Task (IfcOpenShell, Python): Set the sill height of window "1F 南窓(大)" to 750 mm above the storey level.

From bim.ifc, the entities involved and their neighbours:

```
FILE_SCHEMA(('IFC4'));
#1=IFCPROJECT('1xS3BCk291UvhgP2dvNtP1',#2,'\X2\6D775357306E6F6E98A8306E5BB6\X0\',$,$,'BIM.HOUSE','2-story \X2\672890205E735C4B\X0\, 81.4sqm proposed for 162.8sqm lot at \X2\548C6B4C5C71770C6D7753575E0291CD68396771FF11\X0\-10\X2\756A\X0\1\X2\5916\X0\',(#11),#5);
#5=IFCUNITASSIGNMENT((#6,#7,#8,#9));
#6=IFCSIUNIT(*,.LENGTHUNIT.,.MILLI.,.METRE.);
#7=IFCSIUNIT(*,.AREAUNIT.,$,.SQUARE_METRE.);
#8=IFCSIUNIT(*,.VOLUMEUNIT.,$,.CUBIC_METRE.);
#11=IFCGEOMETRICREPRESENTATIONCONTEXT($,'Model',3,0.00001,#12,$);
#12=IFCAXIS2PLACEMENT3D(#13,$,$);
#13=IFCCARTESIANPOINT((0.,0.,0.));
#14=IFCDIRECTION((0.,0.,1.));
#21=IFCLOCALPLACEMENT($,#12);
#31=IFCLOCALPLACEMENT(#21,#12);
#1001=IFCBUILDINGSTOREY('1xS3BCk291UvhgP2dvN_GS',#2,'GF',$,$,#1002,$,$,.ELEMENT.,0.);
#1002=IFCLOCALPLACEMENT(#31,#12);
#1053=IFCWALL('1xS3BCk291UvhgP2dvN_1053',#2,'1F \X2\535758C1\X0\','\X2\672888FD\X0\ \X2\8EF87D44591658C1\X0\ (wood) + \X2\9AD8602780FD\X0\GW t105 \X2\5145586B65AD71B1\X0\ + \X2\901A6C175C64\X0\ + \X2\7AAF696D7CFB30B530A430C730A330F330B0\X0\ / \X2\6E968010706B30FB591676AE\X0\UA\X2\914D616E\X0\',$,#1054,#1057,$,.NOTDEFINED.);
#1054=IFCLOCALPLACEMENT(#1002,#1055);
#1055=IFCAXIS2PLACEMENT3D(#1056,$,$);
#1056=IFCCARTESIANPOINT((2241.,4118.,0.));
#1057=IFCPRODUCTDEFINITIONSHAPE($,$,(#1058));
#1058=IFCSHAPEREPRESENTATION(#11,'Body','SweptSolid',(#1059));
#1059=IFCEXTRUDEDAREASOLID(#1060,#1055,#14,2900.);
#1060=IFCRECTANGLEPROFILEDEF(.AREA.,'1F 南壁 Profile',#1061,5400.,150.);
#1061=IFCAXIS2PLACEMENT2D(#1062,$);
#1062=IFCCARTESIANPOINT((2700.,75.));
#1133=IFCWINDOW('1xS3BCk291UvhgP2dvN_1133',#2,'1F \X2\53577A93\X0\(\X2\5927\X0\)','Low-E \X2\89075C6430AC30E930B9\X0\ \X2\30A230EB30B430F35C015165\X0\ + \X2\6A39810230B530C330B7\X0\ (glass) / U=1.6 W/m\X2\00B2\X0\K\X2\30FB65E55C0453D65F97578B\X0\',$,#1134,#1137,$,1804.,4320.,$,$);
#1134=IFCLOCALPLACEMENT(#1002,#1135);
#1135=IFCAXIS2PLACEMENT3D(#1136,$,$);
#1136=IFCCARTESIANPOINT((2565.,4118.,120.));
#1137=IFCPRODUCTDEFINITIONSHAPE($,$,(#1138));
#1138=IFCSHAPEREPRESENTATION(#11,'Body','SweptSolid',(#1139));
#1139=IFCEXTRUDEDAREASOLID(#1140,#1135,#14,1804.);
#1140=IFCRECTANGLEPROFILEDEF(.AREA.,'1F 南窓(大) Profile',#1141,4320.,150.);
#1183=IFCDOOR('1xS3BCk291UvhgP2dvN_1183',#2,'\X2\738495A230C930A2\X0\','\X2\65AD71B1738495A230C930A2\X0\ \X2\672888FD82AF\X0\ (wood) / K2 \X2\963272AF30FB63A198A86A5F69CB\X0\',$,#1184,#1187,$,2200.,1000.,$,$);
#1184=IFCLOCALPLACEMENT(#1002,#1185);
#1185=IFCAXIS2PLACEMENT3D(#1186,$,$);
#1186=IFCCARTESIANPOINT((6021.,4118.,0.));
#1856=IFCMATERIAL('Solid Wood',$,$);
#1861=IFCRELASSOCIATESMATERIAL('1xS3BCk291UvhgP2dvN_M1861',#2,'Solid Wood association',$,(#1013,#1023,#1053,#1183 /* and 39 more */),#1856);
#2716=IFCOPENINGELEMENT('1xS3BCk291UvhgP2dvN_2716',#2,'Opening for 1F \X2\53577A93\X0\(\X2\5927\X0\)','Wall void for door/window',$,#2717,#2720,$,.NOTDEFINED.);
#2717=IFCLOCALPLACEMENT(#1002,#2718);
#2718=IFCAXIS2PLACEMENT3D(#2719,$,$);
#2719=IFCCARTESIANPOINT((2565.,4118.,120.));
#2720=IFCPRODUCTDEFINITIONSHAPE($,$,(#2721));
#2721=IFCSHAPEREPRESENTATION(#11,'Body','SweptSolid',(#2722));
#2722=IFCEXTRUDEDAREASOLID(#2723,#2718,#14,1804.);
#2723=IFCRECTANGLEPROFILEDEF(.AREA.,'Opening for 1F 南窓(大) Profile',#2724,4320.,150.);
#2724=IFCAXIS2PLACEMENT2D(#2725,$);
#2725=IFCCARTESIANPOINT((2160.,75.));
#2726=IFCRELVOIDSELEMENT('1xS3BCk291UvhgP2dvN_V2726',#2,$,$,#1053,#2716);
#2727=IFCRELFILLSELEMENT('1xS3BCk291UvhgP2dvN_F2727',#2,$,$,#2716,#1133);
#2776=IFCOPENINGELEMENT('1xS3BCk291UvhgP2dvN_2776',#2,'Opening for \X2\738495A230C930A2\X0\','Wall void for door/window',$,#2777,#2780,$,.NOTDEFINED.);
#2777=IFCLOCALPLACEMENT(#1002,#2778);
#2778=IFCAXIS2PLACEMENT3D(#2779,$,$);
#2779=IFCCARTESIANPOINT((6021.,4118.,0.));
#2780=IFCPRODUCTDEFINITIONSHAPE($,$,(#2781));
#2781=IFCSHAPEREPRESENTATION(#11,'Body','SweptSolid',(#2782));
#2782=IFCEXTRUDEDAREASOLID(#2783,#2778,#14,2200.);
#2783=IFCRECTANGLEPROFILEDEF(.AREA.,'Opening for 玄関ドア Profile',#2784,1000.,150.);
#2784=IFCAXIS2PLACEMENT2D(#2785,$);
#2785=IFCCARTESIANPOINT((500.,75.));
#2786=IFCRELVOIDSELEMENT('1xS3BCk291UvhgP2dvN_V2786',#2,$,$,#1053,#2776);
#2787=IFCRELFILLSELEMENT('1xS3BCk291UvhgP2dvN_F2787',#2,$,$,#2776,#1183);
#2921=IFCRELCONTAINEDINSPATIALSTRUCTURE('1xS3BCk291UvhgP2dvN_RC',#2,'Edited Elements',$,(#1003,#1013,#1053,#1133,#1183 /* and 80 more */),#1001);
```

```python
import numpy as np
import ifcopenshell
import ifcopenshell.api.geometry
import ifcopenshell.geom
import ifcopenshell.util.element
import ifcopenshell.util.placement
import ifcopenshell.util.shape
import ifcopenshell.util.unit

model = ifcopenshell.open("bim.ifc")
unit_scale = ifcopenshell.util.unit.calculate_unit_scale(model)

window = model.by_guid("1xS3BCk291UvhgP2dvN_1133")
opening = window.FillsVoids[0].RelatingOpeningElement
storey = ifcopenshell.util.element.get_container(window, ifc_class="IfcBuildingStorey")
level = ifcopenshell.util.placement.get_local_placement(storey.ObjectPlacement)[2, 3]

# The opening's origin need not be at the sill, so measure its lowest point.
shape = ifcopenshell.geom.create_shape(ifcopenshell.geom.settings(), opening)
bottom = ifcopenshell.util.shape.get_shape_bottom_elevation(shape, shape.geometry) / unit_scale
dz = level + 0.75 / unit_scale - bottom

shift = np.array([0.0, 0.0, dz])
# The window is not placed relative to its opening, so move both.
for product in (opening, window):
    matrix = ifcopenshell.util.placement.get_local_placement(product.ObjectPlacement)
    matrix[:3, 3] += shift
    ifcopenshell.api.geometry.edit_object_placement(model, product=product, matrix=matrix, is_si=False)

print(f"moved by {dz * unit_scale:+.3f} m")

model.write("bim_v2.ifc")
```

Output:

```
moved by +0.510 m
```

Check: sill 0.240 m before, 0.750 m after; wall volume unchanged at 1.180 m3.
